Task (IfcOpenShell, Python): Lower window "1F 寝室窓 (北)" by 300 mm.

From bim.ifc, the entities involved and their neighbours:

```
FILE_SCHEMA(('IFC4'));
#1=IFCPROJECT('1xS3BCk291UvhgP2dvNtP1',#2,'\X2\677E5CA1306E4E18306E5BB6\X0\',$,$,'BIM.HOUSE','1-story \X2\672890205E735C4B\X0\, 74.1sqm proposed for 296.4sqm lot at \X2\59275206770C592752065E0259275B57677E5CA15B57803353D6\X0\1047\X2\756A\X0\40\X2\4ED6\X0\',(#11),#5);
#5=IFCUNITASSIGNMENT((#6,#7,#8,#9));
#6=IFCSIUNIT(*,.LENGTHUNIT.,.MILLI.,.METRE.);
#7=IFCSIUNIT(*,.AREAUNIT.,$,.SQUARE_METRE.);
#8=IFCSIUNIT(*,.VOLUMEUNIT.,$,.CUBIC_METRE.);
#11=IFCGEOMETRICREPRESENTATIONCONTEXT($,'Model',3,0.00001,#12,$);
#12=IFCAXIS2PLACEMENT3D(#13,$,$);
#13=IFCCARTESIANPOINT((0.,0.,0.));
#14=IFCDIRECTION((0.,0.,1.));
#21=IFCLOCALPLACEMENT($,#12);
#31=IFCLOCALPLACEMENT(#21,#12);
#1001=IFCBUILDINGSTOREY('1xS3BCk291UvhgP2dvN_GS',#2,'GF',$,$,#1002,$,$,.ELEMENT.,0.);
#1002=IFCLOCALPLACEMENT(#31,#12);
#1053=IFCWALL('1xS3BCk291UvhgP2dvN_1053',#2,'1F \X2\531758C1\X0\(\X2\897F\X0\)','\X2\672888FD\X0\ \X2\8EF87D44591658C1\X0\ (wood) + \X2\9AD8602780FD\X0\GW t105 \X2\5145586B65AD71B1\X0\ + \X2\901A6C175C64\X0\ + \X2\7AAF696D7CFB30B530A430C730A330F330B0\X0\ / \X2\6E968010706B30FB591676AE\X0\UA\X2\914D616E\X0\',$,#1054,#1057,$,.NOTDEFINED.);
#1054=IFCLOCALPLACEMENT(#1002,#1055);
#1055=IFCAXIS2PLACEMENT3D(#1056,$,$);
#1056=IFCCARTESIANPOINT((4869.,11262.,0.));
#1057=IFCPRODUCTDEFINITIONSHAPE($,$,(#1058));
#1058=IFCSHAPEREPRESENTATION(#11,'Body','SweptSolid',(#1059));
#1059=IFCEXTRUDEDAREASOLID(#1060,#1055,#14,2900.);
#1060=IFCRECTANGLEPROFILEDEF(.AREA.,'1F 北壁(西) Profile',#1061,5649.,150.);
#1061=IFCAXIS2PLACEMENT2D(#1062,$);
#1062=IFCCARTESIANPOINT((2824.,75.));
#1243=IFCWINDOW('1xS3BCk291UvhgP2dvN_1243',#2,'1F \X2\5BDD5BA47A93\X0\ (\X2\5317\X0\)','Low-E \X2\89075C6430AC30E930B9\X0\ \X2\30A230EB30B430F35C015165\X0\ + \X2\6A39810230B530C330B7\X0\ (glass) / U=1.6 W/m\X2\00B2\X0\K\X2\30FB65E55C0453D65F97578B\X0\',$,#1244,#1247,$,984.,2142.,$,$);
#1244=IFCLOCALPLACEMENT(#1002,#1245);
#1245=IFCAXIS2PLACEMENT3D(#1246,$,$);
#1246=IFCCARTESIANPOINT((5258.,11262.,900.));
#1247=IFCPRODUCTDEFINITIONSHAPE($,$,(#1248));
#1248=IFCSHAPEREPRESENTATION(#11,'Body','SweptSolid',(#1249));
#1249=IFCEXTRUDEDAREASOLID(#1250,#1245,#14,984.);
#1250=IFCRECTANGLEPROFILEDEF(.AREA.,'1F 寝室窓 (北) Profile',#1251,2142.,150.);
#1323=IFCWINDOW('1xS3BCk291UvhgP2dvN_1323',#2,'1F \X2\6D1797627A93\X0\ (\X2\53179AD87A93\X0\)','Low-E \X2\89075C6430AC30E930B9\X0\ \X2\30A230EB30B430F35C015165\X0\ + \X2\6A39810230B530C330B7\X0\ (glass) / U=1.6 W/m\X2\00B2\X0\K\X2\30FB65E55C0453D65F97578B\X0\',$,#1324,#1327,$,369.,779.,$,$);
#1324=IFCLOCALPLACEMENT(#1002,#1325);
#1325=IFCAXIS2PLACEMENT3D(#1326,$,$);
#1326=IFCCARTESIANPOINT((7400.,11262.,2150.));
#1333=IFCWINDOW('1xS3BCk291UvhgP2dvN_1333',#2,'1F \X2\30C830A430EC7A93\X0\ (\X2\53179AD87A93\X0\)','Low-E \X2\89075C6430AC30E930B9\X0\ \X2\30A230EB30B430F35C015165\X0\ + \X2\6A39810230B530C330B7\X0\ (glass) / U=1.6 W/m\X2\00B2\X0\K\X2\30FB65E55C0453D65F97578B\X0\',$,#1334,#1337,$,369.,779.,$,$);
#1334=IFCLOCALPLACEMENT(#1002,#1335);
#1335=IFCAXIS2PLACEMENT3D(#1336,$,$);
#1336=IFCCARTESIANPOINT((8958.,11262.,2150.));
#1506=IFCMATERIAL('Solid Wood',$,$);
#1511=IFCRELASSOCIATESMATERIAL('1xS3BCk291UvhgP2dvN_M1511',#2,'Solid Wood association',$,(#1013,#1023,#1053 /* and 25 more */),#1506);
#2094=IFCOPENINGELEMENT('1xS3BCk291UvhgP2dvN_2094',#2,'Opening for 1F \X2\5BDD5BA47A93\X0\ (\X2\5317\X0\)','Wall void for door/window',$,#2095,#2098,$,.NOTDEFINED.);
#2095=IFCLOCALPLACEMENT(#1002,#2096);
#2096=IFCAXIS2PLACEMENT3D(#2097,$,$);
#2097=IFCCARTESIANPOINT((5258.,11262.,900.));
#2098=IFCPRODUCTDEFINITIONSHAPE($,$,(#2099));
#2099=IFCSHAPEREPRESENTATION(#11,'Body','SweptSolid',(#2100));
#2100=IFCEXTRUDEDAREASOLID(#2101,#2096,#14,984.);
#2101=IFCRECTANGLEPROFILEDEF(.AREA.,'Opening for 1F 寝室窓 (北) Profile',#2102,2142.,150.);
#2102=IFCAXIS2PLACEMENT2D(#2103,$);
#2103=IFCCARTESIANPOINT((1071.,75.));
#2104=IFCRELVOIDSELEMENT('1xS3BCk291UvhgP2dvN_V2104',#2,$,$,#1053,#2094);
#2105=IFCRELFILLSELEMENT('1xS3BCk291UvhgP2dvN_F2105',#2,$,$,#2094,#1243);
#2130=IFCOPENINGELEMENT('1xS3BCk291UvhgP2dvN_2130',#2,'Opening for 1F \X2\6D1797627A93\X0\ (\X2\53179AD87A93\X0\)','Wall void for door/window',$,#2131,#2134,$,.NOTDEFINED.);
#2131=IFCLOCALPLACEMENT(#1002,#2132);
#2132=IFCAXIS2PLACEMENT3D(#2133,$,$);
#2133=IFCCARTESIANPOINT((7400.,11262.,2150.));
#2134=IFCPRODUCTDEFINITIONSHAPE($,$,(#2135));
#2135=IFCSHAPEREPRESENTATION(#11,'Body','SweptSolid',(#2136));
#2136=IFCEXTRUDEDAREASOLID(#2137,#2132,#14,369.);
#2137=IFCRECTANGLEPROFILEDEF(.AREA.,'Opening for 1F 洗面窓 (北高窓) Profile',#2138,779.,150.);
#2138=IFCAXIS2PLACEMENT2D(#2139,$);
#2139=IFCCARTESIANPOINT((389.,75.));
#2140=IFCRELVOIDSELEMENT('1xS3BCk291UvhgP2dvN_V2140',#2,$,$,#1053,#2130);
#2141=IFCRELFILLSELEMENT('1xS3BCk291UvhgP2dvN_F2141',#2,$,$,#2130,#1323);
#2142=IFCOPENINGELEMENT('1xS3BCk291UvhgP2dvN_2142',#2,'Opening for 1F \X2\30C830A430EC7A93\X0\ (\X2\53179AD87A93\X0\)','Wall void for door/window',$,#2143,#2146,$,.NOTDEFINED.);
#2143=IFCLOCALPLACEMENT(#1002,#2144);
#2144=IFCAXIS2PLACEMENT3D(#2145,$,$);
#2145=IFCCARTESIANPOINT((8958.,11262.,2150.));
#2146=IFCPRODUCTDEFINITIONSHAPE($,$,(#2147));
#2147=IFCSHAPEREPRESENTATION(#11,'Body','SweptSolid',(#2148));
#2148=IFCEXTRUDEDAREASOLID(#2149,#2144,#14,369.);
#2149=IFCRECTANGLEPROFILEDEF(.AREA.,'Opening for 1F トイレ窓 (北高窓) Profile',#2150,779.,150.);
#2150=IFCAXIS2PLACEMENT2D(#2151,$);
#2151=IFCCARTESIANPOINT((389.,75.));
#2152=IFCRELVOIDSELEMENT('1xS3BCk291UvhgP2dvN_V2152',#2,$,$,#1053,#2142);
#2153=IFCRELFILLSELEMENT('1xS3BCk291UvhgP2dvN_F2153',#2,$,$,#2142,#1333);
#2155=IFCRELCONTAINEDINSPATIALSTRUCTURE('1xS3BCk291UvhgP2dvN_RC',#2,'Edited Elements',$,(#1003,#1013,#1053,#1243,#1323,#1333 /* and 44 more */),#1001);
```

```python
import numpy as np
import ifcopenshell
import ifcopenshell.api.geometry
import ifcopenshell.util.placement
import ifcopenshell.util.unit

model = ifcopenshell.open("bim.ifc")
unit_scale = ifcopenshell.util.unit.calculate_unit_scale(model)

window = model.by_guid("1xS3BCk291UvhgP2dvN_1243")
opening = window.FillsVoids[0].RelatingOpeningElement
dz = -0.3 / unit_scale

shift = np.array([0.0, 0.0, dz])
# The window is not placed relative to its opening, so move both.
for product in (opening, window):
    matrix = ifcopenshell.util.placement.get_local_placement(product.ObjectPlacement)
    matrix[:3, 3] += shift
    ifcopenshell.api.geometry.edit_object_placement(model, product=product, matrix=matrix, is_si=False)

print(f"moved by {dz * unit_scale:+.3f} m")

model.write("bim_v2.ifc")
```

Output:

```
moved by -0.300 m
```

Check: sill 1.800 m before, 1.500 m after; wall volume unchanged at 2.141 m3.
